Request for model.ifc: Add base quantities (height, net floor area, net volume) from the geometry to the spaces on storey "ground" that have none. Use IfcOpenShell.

First a look at what the model holds.

```python
import ifcopenshell
import ifcopenshell.util.element
import ifcopenshell.util.unit

model = ifcopenshell.open("model.ifc")
print(model.schema)
for unit_type in ("LENGTHUNIT", "AREAUNIT", "VOLUMEUNIT"):
    print(unit_type, ifcopenshell.util.unit.calculate_unit_scale(model, unit_type))
storey = next(s for s in model.by_type("IfcBuildingStorey") if s.Name == "ground")
spaces = [e for e in ifcopenshell.util.element.get_decomposition(storey) if e.is_a("IfcSpace")]
for e in sorted(spaces, key=lambda e: e.id()):
    print(e.id(), e.is_a(), e.Name, list(ifcopenshell.util.element.get_psets(e, qtos_only=True)), sep=" | ")
```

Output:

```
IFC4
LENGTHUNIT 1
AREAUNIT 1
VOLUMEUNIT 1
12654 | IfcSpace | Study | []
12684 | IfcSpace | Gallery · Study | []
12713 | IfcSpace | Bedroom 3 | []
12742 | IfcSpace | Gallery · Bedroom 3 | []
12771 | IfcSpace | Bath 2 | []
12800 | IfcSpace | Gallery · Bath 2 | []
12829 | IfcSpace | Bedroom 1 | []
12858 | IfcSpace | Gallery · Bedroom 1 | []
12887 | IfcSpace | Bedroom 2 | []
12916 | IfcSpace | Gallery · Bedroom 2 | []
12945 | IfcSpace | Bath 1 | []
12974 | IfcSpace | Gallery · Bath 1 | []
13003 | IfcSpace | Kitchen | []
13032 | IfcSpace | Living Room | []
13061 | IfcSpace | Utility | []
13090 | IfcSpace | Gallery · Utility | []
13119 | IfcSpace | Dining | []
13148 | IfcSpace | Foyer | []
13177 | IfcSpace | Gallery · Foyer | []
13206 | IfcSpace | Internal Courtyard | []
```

```python
import ifcopenshell
import ifcopenshell.api.pset
import ifcopenshell.geom
import ifcopenshell.util.element
import ifcopenshell.util.shape
import ifcopenshell.util.unit

model = ifcopenshell.open("model.ifc")
unit_scale = ifcopenshell.util.unit.calculate_unit_scale(model)
area_scale = ifcopenshell.util.unit.calculate_unit_scale(model, "AREAUNIT")
volume_scale = ifcopenshell.util.unit.calculate_unit_scale(model, "VOLUMEUNIT")
settings = ifcopenshell.geom.settings()

storey = next(s for s in model.by_type("IfcBuildingStorey") if s.Name == "ground")
spaces = [e for e in ifcopenshell.util.element.get_decomposition(storey) if e.is_a("IfcSpace")]

for e in sorted(spaces, key=lambda e: e.id()):
    if ifcopenshell.util.element.get_psets(e, qtos_only=True, should_inherit=False):
        continue
    # Geometry comes back in metres, in the element's own axes.
    shape = ifcopenshell.geom.create_shape(settings, e)
    values = {
        "Height": ifcopenshell.util.shape.get_z(shape.geometry) / unit_scale,
        "NetFloorArea": ifcopenshell.util.shape.get_footprint_area(shape.geometry) / area_scale,
        "NetVolume": ifcopenshell.util.shape.get_volume(shape.geometry) / volume_scale,
    }
    qto = ifcopenshell.api.pset.add_qto(model, product=e, name="Qto_SpaceBaseQuantities")
    ifcopenshell.api.pset.edit_qto(model, qto=qto, properties=values)
    print(e.id(), {k: round(v, 3) for k, v in values.items()})

model.write("model_v2.ifc")
```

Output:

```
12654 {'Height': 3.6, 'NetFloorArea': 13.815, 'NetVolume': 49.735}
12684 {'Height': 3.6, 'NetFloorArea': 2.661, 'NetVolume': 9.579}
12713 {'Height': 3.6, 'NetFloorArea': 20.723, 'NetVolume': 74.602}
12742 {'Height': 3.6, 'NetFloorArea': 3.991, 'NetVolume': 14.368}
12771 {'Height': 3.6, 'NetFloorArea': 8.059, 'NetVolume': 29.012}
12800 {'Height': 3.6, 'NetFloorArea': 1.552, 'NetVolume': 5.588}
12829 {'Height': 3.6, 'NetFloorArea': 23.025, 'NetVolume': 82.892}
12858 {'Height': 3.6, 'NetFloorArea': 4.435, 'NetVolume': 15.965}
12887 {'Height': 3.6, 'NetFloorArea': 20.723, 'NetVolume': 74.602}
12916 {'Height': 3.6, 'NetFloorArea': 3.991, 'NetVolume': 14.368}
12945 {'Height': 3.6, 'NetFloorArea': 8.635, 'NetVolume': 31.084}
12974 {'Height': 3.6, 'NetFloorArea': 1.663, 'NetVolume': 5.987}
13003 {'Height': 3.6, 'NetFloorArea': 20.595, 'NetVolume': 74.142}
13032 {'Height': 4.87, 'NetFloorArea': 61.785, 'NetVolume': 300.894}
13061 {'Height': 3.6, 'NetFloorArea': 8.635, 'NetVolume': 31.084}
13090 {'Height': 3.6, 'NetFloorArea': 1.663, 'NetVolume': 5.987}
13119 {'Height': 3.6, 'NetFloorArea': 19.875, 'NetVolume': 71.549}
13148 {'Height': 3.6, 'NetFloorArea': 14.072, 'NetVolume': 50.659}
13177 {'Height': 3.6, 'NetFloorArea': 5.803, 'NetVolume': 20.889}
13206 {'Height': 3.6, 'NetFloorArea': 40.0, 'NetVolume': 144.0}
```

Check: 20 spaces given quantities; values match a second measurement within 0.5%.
